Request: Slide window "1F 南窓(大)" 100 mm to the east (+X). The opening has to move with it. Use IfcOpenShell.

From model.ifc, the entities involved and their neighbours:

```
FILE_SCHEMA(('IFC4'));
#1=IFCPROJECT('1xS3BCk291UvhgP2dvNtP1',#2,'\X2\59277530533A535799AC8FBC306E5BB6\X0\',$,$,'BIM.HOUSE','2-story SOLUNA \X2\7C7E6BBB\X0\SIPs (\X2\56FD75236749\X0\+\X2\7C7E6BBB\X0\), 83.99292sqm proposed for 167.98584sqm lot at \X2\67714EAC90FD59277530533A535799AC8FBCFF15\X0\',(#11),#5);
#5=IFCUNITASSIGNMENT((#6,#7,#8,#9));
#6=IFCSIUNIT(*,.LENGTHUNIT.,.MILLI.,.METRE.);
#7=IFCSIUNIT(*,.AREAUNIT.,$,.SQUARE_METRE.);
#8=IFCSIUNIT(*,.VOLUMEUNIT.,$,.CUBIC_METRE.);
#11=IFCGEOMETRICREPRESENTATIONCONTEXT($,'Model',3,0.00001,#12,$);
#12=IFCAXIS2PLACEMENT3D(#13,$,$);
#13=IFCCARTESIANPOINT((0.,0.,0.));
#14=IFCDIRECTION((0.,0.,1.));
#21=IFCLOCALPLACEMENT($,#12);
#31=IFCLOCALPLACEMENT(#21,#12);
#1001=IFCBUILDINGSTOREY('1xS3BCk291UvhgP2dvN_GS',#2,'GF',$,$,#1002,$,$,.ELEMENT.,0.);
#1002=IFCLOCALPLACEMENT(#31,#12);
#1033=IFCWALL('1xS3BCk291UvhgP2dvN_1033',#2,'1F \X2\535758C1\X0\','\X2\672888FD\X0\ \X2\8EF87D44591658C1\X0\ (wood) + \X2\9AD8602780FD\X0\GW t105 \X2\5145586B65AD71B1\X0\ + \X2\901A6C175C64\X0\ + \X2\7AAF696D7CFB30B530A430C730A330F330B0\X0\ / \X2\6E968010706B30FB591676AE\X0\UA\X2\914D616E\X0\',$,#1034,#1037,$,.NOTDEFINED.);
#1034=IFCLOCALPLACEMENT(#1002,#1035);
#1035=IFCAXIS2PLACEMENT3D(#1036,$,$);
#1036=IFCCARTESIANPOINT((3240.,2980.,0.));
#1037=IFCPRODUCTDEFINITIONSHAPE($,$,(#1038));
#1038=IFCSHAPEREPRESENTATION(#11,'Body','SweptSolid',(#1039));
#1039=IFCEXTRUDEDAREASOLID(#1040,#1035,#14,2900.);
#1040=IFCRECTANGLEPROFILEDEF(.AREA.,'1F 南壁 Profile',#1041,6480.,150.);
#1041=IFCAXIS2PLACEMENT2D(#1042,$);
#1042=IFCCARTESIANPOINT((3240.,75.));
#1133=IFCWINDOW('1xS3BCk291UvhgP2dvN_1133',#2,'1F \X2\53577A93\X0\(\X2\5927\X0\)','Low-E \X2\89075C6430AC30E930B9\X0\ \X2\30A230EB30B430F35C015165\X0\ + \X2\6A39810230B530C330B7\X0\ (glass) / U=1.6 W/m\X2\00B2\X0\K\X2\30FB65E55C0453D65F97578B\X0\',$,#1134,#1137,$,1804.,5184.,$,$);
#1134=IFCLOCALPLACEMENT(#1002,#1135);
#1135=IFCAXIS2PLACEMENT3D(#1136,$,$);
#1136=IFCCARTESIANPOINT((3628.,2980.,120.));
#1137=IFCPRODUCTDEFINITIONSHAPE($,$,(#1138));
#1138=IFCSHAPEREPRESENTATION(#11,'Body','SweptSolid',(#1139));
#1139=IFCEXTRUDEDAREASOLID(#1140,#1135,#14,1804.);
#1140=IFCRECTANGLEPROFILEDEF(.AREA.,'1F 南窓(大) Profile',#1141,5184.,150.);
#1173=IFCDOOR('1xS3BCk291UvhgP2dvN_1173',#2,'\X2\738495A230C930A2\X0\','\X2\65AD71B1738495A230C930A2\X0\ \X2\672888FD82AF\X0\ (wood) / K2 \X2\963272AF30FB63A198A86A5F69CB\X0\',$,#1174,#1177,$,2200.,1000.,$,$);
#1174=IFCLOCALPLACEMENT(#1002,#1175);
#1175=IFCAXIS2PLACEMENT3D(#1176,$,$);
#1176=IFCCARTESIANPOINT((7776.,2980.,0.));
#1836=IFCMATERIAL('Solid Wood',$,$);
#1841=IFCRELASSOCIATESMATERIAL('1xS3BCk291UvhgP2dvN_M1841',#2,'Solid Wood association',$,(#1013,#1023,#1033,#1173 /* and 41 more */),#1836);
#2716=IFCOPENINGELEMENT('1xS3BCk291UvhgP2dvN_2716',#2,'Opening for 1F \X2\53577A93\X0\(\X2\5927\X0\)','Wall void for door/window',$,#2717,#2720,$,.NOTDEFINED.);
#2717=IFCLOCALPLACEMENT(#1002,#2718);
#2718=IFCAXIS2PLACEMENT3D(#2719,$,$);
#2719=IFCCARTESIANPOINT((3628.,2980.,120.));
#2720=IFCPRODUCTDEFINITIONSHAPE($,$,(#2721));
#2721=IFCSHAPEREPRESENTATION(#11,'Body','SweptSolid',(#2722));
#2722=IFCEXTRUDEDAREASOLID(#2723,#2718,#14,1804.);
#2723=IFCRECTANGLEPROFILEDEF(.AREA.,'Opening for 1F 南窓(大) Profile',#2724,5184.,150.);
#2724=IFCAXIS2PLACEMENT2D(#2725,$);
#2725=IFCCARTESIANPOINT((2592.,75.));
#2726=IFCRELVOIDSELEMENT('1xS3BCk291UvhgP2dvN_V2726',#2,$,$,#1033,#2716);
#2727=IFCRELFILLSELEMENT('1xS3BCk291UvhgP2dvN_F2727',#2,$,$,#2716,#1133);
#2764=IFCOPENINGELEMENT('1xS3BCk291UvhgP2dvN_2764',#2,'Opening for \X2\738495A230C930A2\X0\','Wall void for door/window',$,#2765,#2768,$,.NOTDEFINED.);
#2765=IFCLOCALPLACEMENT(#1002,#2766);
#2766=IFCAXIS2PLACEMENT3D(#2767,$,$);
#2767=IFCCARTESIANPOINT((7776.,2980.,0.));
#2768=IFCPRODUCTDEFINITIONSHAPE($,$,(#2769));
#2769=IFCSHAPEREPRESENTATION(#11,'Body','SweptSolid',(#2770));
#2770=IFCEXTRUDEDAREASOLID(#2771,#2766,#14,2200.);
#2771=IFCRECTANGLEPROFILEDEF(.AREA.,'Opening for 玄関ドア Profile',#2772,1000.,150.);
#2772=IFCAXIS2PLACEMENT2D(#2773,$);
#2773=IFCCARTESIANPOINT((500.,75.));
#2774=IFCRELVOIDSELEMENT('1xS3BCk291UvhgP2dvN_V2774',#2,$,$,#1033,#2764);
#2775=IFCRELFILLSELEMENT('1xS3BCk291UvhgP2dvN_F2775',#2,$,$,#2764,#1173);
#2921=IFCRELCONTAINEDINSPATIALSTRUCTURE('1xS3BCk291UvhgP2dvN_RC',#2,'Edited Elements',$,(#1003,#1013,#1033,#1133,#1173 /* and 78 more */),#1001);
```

```python
import ifcopenshell
import ifcopenshell.api.geometry
import ifcopenshell.util.placement

model = ifcopenshell.open("model.ifc")

window = model.by_id(1133)
opening = window.FillsVoids[0].RelatingOpeningElement
wall = opening.VoidsElements[0].RelatingBuildingElement

wall_matrix = ifcopenshell.util.placement.get_local_placement(wall.ObjectPlacement)
shift = wall_matrix[:3, 0] * 100.0
before = ifcopenshell.util.placement.get_local_placement(window.ObjectPlacement)[:3, 3].copy()

# The window is not placed relative to its opening, so move both.
for product in (opening, window):
    matrix = ifcopenshell.util.placement.get_local_placement(product.ObjectPlacement)
    matrix[:3, 3] += shift
    ifcopenshell.api.geometry.edit_object_placement(model, product=product, matrix=matrix, is_si=False)

after = ifcopenshell.util.placement.get_local_placement(window.ObjectPlacement)[:3, 3]
print("window moved by", (after - before).round(3) + 0.0)

model.write("model-out.ifc")
```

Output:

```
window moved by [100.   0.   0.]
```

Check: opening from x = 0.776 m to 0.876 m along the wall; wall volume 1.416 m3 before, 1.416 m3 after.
